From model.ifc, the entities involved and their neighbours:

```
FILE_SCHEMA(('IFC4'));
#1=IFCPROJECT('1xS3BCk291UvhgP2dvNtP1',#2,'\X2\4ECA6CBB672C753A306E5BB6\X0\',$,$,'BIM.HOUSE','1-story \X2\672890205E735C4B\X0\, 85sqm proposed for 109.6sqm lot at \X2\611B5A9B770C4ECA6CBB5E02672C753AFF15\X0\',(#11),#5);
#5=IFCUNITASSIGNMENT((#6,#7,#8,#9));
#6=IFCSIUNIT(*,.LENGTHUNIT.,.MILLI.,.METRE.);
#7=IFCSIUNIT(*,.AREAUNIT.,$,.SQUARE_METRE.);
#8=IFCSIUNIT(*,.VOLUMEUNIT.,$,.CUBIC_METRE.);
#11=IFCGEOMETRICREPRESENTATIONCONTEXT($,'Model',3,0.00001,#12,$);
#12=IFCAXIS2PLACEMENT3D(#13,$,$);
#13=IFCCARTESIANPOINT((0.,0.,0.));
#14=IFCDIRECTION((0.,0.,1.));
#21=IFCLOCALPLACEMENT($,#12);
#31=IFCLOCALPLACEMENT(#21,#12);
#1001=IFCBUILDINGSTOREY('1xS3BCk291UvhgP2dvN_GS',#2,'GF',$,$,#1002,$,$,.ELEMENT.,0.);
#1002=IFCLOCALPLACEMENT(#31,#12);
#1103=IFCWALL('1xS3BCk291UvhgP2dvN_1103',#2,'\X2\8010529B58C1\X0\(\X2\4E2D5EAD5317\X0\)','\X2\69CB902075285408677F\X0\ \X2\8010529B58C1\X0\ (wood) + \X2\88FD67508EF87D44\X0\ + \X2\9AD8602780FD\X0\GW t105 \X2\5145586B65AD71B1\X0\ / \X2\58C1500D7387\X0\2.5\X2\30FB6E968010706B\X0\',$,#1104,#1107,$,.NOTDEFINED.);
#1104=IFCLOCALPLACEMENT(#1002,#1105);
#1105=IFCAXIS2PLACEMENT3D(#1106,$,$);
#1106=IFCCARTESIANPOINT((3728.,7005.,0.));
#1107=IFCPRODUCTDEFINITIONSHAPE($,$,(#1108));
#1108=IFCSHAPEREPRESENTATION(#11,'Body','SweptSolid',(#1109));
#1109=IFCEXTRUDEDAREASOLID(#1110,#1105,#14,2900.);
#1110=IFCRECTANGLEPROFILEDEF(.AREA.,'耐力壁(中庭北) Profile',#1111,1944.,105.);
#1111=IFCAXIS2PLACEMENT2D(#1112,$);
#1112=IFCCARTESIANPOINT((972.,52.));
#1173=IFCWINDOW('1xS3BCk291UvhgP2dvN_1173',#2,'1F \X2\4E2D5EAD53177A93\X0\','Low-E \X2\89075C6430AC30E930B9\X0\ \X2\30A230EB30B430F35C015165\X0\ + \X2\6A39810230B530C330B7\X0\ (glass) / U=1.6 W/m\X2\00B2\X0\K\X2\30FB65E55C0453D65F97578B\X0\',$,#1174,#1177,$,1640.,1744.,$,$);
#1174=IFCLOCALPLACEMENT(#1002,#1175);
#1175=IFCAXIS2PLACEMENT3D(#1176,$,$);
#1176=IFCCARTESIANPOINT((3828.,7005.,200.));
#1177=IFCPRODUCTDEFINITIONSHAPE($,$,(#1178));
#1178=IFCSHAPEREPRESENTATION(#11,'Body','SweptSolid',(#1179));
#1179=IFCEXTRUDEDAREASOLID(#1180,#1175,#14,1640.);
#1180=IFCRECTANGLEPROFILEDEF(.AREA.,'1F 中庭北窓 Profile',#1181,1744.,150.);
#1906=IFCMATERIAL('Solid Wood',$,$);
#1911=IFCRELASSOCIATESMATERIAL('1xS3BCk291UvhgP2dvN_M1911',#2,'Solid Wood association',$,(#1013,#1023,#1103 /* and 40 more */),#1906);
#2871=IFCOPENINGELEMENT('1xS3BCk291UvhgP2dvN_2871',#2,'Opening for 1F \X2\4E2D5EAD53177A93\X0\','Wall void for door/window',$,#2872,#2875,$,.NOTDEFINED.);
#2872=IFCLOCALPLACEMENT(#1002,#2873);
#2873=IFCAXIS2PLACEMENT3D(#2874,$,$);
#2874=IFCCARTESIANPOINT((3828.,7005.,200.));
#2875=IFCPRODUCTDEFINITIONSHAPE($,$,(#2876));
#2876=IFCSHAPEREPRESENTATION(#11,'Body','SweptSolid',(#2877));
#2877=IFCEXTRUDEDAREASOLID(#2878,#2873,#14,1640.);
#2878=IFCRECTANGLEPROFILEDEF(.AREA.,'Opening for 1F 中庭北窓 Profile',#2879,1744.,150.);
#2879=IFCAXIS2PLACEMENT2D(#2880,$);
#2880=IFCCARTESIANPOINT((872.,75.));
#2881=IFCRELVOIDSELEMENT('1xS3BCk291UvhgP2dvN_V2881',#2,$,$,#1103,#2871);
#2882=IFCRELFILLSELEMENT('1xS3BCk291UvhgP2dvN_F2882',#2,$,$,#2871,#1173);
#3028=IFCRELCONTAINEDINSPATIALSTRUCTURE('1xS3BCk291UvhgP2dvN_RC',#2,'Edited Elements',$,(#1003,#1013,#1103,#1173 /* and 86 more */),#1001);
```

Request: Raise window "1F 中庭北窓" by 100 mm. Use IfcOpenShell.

```python
import numpy as np
import ifcopenshell
import ifcopenshell.api.geometry
import ifcopenshell.util.placement
import ifcopenshell.util.unit

model = ifcopenshell.open("model.ifc")
unit_scale = ifcopenshell.util.unit.calculate_unit_scale(model)

window = model.by_guid("1xS3BCk291UvhgP2dvN_1173")
opening = window.FillsVoids[0].RelatingOpeningElement
dz = 100.0

shift = np.array([0.0, 0.0, dz])
# The window is not placed relative to its opening, so move both.
for product in (opening, window):
    matrix = ifcopenshell.util.placement.get_local_placement(product.ObjectPlacement)
    matrix[:3, 3] += shift
    ifcopenshell.api.geometry.edit_object_placement(model, product=product, matrix=matrix, is_si=False)

print(f"moved by {dz * unit_scale:+.3f} m")

model.write("model-out.ifc")
```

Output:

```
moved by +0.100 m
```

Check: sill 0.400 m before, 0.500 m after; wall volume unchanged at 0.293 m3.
